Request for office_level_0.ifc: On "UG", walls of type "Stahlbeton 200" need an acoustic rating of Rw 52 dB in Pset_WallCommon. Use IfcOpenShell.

First a look at what the model holds.

```python
import ifcopenshell
import ifcopenshell.util.element

model = ifcopenshell.open("office_level_0.ifc")
print(model.schema)
storey = next(s for s in model.by_type("IfcBuildingStorey") if s.Name == "UG")
walls = [e for e in ifcopenshell.util.element.get_decomposition(storey) if e.is_a("IfcWall")]
seen = {}
for e in walls:
    element_type = ifcopenshell.util.element.get_type(e)
    key = (element_type.Name if element_type != e and element_type else None, ifcopenshell.util.element.get_pset(e, "Pset_WallCommon", "AcousticRating"))
    seen[key] = seen.get(key, 0) + 1
for (name, value), count in sorted(seen.items(), key=str):
    print(count, "x", name, "|", value)
```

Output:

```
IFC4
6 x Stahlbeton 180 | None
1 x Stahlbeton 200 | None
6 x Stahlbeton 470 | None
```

```python
import ifcopenshell
import ifcopenshell.api.pset
import ifcopenshell.util.element

model = ifcopenshell.open("office_level_0.ifc")

storey = next(s for s in model.by_type("IfcBuildingStorey") if s.Name == "UG")
walls = [e for e in ifcopenshell.util.element.get_decomposition(storey) if e.is_a("IfcWall")]

count = 0
for e in walls:
    element_type = ifcopenshell.util.element.get_type(e)
    if element_type in (None, e) or element_type.Name != "Stahlbeton 200":
        continue
    # add_pset returns the element's existing set when there is one.
    pset = ifcopenshell.api.pset.add_pset(model, product=e, name="Pset_WallCommon")
    ifcopenshell.api.pset.edit_pset(model, pset=pset, properties={"AcousticRating": "Rw 52 dB"})
    count += 1

print(count, "walls updated")

model.write("office_level_0_edited.ifc")
```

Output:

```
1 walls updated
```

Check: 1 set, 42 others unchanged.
